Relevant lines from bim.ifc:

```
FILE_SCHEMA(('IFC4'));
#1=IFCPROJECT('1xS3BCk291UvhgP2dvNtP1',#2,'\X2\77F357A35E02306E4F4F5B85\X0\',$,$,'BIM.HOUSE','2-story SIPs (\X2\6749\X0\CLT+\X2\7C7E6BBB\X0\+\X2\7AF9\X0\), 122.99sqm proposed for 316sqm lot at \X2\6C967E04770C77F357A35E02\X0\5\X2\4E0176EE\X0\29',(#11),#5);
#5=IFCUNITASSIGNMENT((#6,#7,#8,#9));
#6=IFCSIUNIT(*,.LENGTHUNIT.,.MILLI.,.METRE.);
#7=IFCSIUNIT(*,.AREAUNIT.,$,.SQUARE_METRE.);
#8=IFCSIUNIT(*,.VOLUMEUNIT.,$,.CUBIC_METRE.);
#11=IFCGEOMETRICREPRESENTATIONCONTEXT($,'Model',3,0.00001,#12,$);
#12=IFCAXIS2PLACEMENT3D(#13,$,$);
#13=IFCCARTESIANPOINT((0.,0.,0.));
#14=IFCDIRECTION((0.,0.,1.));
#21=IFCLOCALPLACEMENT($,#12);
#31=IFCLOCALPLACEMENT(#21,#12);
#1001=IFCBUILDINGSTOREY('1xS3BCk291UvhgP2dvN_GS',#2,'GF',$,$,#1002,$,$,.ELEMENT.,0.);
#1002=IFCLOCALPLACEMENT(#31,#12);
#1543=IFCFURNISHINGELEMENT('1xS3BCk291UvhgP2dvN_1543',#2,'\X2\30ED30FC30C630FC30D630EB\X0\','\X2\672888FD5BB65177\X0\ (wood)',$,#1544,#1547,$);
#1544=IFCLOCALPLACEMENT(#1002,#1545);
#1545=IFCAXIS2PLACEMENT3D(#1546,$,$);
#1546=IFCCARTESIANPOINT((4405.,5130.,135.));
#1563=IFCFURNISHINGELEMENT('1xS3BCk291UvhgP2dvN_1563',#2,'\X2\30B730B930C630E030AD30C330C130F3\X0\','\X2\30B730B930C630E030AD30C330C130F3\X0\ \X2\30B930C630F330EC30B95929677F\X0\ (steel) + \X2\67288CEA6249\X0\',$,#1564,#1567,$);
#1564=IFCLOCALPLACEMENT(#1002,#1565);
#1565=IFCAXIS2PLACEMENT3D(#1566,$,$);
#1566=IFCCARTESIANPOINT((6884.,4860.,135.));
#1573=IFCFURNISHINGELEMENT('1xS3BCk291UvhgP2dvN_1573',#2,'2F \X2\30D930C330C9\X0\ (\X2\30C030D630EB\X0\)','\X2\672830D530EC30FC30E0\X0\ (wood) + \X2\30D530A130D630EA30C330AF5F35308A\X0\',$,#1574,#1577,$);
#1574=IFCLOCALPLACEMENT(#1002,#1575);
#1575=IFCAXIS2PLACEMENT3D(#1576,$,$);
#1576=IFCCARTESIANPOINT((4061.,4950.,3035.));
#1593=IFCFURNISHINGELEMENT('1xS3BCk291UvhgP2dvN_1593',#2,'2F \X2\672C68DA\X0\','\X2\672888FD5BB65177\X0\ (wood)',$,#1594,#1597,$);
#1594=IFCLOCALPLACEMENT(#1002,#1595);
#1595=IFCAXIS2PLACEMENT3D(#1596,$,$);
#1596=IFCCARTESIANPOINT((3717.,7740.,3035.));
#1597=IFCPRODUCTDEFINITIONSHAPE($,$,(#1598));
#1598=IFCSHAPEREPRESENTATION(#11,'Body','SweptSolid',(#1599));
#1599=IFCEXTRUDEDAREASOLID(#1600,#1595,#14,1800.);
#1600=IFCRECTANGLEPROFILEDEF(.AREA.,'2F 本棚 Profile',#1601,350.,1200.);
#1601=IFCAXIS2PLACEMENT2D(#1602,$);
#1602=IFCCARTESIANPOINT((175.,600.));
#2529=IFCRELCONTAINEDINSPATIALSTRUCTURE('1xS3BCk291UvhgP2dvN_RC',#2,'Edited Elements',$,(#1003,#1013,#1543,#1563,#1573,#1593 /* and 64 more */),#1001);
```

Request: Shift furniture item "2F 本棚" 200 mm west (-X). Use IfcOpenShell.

```python
import ifcopenshell
import ifcopenshell.api.geometry
import ifcopenshell.util.placement
import ifcopenshell.util.unit

model = ifcopenshell.open("bim.ifc")
unit_scale = ifcopenshell.util.unit.calculate_unit_scale(model)

item = model.by_guid("1xS3BCk291UvhgP2dvN_1593")
matrix = ifcopenshell.util.placement.get_local_placement(item.ObjectPlacement)
matrix[0, 3] -= 0.2 / unit_scale
ifcopenshell.api.geometry.edit_object_placement(model, product=item, matrix=matrix, is_si=False)

print(ifcopenshell.util.placement.get_local_placement(item.ObjectPlacement).round(3) + 0.0)

model.write("bim-out.ifc")
```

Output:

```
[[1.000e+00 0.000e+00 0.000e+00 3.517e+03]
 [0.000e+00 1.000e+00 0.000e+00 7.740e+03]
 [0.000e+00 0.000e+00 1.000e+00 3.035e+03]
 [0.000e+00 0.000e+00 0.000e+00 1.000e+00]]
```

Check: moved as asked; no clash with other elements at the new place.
